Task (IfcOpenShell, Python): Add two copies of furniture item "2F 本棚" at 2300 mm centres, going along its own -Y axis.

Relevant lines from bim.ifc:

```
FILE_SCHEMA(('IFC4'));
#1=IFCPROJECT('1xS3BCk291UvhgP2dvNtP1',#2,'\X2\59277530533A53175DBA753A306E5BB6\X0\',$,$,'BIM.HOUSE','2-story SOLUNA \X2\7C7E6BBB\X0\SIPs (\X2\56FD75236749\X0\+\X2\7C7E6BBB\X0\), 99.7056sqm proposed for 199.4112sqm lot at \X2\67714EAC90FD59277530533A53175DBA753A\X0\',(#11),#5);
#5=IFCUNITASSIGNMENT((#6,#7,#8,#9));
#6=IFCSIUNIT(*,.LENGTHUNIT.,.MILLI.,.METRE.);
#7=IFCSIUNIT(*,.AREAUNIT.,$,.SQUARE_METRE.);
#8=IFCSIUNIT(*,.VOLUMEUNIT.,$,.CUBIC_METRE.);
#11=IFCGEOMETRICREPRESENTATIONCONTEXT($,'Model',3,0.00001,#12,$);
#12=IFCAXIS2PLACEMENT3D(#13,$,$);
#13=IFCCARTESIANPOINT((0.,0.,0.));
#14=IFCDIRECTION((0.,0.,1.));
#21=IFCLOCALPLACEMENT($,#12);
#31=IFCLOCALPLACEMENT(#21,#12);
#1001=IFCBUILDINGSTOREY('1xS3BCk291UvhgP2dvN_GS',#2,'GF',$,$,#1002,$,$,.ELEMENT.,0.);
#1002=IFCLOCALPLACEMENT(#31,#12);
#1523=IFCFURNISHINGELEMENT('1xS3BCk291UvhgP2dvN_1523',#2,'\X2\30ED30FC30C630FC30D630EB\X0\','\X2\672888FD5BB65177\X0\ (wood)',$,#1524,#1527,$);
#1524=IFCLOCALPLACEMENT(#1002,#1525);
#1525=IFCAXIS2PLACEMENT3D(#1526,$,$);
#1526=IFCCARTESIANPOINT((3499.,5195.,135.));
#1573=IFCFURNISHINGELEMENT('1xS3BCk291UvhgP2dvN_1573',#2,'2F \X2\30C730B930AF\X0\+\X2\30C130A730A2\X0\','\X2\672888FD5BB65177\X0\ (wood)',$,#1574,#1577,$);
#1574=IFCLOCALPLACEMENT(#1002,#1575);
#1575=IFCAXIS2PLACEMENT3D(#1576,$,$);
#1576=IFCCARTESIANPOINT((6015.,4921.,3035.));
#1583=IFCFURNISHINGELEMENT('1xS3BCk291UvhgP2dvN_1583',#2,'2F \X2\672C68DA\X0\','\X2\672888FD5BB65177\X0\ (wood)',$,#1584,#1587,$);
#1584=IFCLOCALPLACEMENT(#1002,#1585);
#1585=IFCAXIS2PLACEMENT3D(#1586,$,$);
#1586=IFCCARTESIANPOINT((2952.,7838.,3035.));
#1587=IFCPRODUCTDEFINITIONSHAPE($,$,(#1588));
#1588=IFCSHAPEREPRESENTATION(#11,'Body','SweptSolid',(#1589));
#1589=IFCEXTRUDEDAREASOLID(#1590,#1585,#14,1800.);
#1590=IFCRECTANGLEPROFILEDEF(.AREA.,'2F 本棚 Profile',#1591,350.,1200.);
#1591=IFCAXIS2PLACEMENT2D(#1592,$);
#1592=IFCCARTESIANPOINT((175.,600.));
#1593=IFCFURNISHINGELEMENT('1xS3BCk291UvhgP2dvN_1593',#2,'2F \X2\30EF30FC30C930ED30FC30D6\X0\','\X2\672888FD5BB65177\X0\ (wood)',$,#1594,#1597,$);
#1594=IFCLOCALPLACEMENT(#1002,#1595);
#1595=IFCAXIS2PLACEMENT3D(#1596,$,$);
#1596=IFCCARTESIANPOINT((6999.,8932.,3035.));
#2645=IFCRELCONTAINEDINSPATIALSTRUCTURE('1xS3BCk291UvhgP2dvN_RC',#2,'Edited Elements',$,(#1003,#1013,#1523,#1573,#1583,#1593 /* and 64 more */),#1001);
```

```python
import ifcopenshell
import ifcopenshell.api.geometry
import ifcopenshell.api.root
import ifcopenshell.util.element
import ifcopenshell.util.placement
import ifcopenshell.util.unit

model = ifcopenshell.open("bim.ifc")
unit_scale = ifcopenshell.util.unit.calculate_unit_scale(model)


def reuse_history(source, copy):
    """copy_class also copies each property set's owner history, people and application; keep the originals."""
    for rel in copy.IsDefinedBy:
        if rel.is_a("IfcRelDefinesByProperties") and (history := rel.RelatingPropertyDefinition.OwnerHistory):
            rel.RelatingPropertyDefinition.OwnerHistory = source.OwnerHistory
            ifcopenshell.util.element.remove_deep2(model, history)


source = model.by_guid("1xS3BCk291UvhgP2dvN_1583")
base = ifcopenshell.util.placement.get_local_placement(source.ObjectPlacement)
step = -base[:3, 1] * 2.3 / unit_scale

for i in range(1, 3):
    copy = ifcopenshell.api.root.copy_class(model, product=source)
    copy.Representation = ifcopenshell.util.element.copy_deep(
        model, source.Representation, exclude=["IfcGeometricRepresentationContext", "IfcRepresentationMap"]
    )
    reuse_history(source, copy)
    matrix = base.copy()
    matrix[:3, 3] += i * step
    print("added at", matrix[:3, 3].round(3) + 0.0)
    ifcopenshell.api.geometry.edit_object_placement(model, product=copy, matrix=matrix, is_si=False)

model.write("bim_edited.ifc")
```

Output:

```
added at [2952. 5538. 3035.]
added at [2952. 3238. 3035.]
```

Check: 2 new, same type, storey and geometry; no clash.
